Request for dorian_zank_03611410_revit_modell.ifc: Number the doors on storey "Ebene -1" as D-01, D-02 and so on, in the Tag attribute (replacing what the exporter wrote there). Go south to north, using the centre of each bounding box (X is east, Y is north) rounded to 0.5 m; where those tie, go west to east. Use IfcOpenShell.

First a look at what the model holds.

```python
import ifcopenshell
import ifcopenshell.util.element
import ifcopenshell.util.placement

model = ifcopenshell.open("dorian_zank_03611410_revit_modell.ifc")
print(model.schema)
storey = next(s for s in model.by_type("IfcBuildingStorey") if s.Name == "Ebene -1")
doors = [e for e in ifcopenshell.util.element.get_decomposition(storey) if e.is_a("IfcDoor")]
for e in sorted(doors, key=lambda e: e.id()):
    origin = ifcopenshell.util.placement.get_local_placement(e.ObjectPlacement)[:3, 3]
    print(e.id(), e.Tag, e.Name, origin.round(2) + 0.0, sep=" | ")
```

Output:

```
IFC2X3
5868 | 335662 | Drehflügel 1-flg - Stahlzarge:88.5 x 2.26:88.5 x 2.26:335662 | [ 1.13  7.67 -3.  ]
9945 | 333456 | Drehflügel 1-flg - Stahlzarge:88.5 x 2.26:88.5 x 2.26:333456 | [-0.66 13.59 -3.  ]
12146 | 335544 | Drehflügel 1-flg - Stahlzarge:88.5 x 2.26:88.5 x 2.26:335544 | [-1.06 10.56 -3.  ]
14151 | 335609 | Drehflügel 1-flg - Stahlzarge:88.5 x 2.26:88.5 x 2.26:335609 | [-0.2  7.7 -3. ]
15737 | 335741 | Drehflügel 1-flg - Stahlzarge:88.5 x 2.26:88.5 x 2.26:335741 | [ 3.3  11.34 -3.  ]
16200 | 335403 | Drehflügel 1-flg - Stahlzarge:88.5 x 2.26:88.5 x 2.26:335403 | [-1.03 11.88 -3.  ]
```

```python
import ifcopenshell
import ifcopenshell.geom
import ifcopenshell.util.element
import ifcopenshell.util.shape

model = ifcopenshell.open("dorian_zank_03611410_revit_modell.ifc")
settings = ifcopenshell.geom.settings()
settings.set("use-world-coords", True)


def centre(element):
    shape = ifcopenshell.geom.create_shape(settings, element)
    return ifcopenshell.util.shape.get_bbox_centroid(shape.geometry)


storey = next(s for s in model.by_type("IfcBuildingStorey") if s.Name == "Ebene -1")
doors = [e for e in ifcopenshell.util.element.get_decomposition(storey) if e.is_a("IfcDoor")]

# Insertion points can sit at a corner or the storey origin, so sort by the geometry (in metres).
centres = {e: centre(e) for e in doors}
doors.sort(key=lambda e: (round(centres[e][1] / 0.5), centres[e][0]))

for i, e in enumerate(doors, start=1):
    number = f"D-{i:02d}"
    e.Tag = number
    print(e.id(), number)

model.write("dorian_zank_03611410_revit_modell_rev.ifc")
```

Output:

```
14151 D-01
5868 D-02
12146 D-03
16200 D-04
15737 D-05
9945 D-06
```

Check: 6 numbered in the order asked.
